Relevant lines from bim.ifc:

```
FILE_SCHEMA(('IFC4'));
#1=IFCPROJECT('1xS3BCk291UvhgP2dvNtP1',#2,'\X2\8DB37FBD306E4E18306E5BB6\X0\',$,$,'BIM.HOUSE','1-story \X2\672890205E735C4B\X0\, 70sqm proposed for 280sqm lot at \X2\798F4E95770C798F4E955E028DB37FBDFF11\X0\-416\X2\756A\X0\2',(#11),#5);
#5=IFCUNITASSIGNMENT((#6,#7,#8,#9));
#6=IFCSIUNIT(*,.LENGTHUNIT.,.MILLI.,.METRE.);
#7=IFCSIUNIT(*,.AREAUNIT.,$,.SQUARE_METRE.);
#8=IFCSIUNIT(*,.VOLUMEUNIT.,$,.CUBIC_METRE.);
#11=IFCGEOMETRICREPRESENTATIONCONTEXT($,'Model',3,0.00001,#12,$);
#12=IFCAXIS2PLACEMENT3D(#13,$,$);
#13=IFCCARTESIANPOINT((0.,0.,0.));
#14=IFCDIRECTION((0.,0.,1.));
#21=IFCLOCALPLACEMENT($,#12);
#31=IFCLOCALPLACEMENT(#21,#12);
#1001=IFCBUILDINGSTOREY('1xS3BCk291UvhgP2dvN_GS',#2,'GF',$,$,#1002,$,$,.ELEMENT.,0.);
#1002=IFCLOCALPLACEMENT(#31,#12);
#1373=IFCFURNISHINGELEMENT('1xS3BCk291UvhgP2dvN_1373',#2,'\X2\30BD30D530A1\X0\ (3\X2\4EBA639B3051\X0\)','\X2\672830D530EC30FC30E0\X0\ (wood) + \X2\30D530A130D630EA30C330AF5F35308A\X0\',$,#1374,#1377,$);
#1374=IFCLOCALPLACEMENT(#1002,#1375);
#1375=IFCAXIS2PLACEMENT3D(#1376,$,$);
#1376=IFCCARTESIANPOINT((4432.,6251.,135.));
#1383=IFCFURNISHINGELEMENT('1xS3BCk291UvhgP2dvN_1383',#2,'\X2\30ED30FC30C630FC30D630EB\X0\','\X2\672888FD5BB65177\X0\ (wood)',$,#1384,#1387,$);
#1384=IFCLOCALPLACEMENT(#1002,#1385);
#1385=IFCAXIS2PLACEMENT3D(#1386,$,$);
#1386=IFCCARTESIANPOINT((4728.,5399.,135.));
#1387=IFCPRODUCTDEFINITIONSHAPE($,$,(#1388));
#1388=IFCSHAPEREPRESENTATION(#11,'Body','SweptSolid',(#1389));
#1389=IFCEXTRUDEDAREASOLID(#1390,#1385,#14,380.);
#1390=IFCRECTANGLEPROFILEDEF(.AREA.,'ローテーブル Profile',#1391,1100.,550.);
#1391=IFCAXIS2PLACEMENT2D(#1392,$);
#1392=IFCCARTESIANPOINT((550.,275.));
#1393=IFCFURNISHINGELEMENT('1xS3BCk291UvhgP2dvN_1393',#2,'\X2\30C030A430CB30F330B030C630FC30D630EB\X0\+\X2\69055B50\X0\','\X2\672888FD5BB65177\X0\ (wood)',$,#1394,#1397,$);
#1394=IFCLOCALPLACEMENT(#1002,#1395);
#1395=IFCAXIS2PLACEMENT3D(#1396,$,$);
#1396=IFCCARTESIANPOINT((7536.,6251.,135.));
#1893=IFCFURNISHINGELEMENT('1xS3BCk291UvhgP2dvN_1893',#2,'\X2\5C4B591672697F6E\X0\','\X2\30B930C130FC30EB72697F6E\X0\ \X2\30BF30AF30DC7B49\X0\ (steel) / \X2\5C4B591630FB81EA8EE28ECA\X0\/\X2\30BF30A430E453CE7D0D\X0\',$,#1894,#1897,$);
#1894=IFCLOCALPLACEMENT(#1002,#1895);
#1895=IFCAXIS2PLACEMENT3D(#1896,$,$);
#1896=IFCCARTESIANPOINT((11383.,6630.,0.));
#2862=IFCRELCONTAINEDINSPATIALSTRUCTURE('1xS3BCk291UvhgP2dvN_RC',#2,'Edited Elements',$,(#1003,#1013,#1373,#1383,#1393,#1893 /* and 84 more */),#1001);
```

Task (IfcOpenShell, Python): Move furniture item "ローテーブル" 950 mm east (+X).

```python
import ifcopenshell
import ifcopenshell.api.geometry
import ifcopenshell.util.placement
import ifcopenshell.util.unit

model = ifcopenshell.open("bim.ifc")
unit_scale = ifcopenshell.util.unit.calculate_unit_scale(model)

item = model.by_id(1383)
matrix = ifcopenshell.util.placement.get_local_placement(item.ObjectPlacement)
matrix[0, 3] += 0.95 / unit_scale
ifcopenshell.api.geometry.edit_object_placement(model, product=item, matrix=matrix, is_si=False)

print(ifcopenshell.util.placement.get_local_placement(item.ObjectPlacement).round(3) + 0.0)

model.write("bim-out.ifc")
```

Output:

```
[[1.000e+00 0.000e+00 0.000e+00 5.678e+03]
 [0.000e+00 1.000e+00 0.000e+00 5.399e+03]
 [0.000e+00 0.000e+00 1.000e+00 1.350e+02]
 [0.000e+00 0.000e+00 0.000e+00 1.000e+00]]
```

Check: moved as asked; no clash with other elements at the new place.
